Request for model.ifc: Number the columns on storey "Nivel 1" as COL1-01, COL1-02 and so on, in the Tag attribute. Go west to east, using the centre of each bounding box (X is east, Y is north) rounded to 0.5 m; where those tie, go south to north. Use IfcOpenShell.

First a look at what the model holds.

```python
import ifcopenshell
import ifcopenshell.util.element
import ifcopenshell.util.placement

model = ifcopenshell.open("model.ifc")
print(model.schema)
storey = next(s for s in model.by_type("IfcBuildingStorey") if s.Name == "Nivel 1")
columns = [e for e in ifcopenshell.util.element.get_decomposition(storey) if e.is_a("IfcColumn")]
for e in sorted(columns, key=lambda e: e.id()):
    origin = ifcopenshell.util.placement.get_local_placement(e.ObjectPlacement)[:3, 3]
    print(e.id(), e.Tag, e.Name, origin.round(2) + 0.0, sep=" | ")
```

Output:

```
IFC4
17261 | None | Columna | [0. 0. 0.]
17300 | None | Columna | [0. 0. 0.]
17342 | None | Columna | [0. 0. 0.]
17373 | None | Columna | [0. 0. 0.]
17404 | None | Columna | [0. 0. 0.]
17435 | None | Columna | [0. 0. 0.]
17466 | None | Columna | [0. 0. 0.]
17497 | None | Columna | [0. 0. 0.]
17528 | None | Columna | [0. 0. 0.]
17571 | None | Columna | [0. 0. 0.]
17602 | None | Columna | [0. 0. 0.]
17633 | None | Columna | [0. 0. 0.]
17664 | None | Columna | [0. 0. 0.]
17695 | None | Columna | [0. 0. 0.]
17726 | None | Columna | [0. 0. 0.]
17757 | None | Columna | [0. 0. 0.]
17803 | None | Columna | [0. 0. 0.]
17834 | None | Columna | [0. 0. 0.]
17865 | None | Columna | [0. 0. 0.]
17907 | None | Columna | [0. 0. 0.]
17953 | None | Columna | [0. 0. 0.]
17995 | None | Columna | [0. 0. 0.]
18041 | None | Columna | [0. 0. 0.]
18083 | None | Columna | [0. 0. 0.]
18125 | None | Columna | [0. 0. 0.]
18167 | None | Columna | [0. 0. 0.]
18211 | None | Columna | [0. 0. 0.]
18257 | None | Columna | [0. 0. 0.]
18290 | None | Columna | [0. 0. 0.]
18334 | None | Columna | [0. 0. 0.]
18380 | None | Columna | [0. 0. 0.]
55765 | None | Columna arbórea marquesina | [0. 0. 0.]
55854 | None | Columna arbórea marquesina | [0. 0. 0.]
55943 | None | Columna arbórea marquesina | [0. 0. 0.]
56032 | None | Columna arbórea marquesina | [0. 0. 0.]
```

```python
import ifcopenshell
import ifcopenshell.geom
import ifcopenshell.util.element
import ifcopenshell.util.shape

model = ifcopenshell.open("model.ifc")
settings = ifcopenshell.geom.settings()
settings.set("use-world-coords", True)


def centre(element):
    shape = ifcopenshell.geom.create_shape(settings, element)
    return ifcopenshell.util.shape.get_bbox_centroid(shape.geometry)


storey = next(s for s in model.by_type("IfcBuildingStorey") if s.Name == "Nivel 1")
columns = [e for e in ifcopenshell.util.element.get_decomposition(storey) if e.is_a("IfcColumn")]

# Insertion points can sit at a corner or the storey origin, so sort by the geometry (in metres).
centres = {e: centre(e) for e in columns}
columns.sort(key=lambda e: (round(centres[e][0] / 0.5), centres[e][1]))

for i, e in enumerate(columns, start=1):
    number = f"COL1-{i:02d}"
    e.Tag = number
    print(e.id(), number)

model.write("model_updated.ifc")
```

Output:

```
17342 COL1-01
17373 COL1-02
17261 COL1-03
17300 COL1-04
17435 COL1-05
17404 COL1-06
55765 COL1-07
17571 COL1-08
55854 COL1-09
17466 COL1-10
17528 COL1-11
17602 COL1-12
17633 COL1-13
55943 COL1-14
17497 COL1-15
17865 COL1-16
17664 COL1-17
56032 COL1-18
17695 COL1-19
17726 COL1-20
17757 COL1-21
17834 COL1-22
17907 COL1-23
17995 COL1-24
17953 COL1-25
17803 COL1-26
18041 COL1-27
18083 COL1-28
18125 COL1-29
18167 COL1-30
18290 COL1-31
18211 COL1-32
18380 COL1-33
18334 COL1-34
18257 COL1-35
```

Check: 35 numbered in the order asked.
